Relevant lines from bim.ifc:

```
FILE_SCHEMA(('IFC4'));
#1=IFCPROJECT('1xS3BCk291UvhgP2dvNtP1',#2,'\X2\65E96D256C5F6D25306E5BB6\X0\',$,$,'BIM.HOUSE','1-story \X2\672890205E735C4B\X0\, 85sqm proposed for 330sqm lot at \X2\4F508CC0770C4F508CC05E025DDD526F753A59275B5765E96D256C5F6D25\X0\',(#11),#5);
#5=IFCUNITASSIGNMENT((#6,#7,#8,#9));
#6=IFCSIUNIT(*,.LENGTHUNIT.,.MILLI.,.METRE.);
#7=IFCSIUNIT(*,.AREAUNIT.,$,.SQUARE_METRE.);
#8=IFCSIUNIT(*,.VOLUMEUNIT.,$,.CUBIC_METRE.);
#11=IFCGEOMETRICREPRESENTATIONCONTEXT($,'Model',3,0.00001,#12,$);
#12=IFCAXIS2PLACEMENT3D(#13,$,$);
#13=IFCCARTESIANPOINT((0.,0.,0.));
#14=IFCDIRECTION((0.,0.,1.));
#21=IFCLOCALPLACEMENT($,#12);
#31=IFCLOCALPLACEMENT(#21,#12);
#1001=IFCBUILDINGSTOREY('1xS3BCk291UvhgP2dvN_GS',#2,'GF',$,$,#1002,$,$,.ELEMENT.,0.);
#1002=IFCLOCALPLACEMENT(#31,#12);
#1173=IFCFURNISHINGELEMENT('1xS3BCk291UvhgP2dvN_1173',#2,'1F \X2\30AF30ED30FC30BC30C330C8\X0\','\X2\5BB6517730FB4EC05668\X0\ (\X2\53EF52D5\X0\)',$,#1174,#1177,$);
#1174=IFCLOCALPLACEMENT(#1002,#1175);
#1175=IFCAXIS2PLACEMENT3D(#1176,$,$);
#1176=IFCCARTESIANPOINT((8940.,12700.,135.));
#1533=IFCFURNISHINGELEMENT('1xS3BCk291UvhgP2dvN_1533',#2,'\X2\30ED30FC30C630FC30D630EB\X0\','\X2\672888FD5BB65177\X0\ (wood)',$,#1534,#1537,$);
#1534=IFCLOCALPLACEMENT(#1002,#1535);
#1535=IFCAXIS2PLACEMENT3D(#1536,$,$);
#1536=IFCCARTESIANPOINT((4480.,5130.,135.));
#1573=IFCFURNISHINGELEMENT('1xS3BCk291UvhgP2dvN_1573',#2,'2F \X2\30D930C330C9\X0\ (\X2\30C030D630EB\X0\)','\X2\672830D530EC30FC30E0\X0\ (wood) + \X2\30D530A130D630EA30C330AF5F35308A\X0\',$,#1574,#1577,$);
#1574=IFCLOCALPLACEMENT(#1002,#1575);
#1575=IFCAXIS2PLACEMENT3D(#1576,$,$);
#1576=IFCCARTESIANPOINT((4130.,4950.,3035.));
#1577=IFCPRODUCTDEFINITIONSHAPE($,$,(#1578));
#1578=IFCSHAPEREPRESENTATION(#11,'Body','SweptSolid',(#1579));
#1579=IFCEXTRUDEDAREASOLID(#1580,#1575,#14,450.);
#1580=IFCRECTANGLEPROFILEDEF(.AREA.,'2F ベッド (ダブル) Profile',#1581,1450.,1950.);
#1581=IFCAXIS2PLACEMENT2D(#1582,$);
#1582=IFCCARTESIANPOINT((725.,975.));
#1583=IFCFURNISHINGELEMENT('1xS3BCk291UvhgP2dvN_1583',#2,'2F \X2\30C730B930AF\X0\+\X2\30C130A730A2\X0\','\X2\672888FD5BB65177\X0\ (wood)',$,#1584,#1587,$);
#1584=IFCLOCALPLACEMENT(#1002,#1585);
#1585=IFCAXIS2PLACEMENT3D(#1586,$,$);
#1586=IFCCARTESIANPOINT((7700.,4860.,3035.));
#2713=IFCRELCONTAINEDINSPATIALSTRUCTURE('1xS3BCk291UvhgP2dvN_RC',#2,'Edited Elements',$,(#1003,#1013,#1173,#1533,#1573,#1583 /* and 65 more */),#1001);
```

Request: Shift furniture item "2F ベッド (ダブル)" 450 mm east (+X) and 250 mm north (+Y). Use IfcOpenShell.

```python
import ifcopenshell
import ifcopenshell.api.geometry
import ifcopenshell.util.placement
import ifcopenshell.util.unit

model = ifcopenshell.open("bim.ifc")
unit_scale = ifcopenshell.util.unit.calculate_unit_scale(model)

item = model.by_guid("1xS3BCk291UvhgP2dvN_1573")
matrix = ifcopenshell.util.placement.get_local_placement(item.ObjectPlacement)
matrix[0, 3] += 0.45 / unit_scale
matrix[1, 3] += 0.25 / unit_scale
ifcopenshell.api.geometry.edit_object_placement(model, product=item, matrix=matrix, is_si=False)

print(ifcopenshell.util.placement.get_local_placement(item.ObjectPlacement).round(3) + 0.0)

model.write("bim_edited.ifc")
```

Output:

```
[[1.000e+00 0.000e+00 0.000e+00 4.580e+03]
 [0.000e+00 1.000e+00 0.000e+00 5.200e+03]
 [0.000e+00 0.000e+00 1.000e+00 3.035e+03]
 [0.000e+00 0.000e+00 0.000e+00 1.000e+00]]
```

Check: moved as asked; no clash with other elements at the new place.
